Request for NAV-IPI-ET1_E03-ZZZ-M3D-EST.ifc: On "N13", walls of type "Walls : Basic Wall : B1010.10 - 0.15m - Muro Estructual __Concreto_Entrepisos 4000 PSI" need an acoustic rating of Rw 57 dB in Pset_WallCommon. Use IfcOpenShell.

First a look at what the model holds.

```python
import ifcopenshell
import ifcopenshell.util.element

model = ifcopenshell.open("NAV-IPI-ET1_E03-ZZZ-M3D-EST.ifc")
print(model.schema)
storey = next(s for s in model.by_type("IfcBuildingStorey") if s.Name == "N13")
walls = [e for e in ifcopenshell.util.element.get_decomposition(storey) if e.is_a("IfcWall")]
seen = {}
for e in walls:
    element_type = ifcopenshell.util.element.get_type(e)
    key = (element_type.Name if element_type != e and element_type else None, ifcopenshell.util.element.get_pset(e, "Pset_WallCommon", "AcousticRating"))
    seen[key] = seen.get(key, 0) + 1
for (name, value), count in sorted(seen.items(), key=str):
    print(count, "x", name, "|", value)
```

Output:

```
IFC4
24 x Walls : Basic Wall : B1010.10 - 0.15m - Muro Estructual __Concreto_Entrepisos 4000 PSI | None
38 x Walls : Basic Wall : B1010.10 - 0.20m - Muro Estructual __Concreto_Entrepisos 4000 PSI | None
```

```python
import ifcopenshell
import ifcopenshell.api.pset
import ifcopenshell.util.element

model = ifcopenshell.open("NAV-IPI-ET1_E03-ZZZ-M3D-EST.ifc")

storey = next(s for s in model.by_type("IfcBuildingStorey") if s.Name == "N13")
walls = [e for e in ifcopenshell.util.element.get_decomposition(storey) if e.is_a("IfcWall")]

count = 0
for e in walls:
    element_type = ifcopenshell.util.element.get_type(e)
    if element_type in (None, e) or element_type.Name != "Walls : Basic Wall : B1010.10 - 0.15m - Muro Estructual __Concreto_Entrepisos 4000 PSI":
        continue
    # add_pset returns the element's existing set when there is one.
    pset = ifcopenshell.api.pset.add_pset(model, product=e, name="Pset_WallCommon")
    ifcopenshell.api.pset.edit_pset(model, pset=pset, properties={"AcousticRating": "Rw 57 dB"})
    count += 1

print(count, "walls updated")

model.write("NAV-IPI-ET1_E03-ZZZ-M3D-EST_rev.ifc")
```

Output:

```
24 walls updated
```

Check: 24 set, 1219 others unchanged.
